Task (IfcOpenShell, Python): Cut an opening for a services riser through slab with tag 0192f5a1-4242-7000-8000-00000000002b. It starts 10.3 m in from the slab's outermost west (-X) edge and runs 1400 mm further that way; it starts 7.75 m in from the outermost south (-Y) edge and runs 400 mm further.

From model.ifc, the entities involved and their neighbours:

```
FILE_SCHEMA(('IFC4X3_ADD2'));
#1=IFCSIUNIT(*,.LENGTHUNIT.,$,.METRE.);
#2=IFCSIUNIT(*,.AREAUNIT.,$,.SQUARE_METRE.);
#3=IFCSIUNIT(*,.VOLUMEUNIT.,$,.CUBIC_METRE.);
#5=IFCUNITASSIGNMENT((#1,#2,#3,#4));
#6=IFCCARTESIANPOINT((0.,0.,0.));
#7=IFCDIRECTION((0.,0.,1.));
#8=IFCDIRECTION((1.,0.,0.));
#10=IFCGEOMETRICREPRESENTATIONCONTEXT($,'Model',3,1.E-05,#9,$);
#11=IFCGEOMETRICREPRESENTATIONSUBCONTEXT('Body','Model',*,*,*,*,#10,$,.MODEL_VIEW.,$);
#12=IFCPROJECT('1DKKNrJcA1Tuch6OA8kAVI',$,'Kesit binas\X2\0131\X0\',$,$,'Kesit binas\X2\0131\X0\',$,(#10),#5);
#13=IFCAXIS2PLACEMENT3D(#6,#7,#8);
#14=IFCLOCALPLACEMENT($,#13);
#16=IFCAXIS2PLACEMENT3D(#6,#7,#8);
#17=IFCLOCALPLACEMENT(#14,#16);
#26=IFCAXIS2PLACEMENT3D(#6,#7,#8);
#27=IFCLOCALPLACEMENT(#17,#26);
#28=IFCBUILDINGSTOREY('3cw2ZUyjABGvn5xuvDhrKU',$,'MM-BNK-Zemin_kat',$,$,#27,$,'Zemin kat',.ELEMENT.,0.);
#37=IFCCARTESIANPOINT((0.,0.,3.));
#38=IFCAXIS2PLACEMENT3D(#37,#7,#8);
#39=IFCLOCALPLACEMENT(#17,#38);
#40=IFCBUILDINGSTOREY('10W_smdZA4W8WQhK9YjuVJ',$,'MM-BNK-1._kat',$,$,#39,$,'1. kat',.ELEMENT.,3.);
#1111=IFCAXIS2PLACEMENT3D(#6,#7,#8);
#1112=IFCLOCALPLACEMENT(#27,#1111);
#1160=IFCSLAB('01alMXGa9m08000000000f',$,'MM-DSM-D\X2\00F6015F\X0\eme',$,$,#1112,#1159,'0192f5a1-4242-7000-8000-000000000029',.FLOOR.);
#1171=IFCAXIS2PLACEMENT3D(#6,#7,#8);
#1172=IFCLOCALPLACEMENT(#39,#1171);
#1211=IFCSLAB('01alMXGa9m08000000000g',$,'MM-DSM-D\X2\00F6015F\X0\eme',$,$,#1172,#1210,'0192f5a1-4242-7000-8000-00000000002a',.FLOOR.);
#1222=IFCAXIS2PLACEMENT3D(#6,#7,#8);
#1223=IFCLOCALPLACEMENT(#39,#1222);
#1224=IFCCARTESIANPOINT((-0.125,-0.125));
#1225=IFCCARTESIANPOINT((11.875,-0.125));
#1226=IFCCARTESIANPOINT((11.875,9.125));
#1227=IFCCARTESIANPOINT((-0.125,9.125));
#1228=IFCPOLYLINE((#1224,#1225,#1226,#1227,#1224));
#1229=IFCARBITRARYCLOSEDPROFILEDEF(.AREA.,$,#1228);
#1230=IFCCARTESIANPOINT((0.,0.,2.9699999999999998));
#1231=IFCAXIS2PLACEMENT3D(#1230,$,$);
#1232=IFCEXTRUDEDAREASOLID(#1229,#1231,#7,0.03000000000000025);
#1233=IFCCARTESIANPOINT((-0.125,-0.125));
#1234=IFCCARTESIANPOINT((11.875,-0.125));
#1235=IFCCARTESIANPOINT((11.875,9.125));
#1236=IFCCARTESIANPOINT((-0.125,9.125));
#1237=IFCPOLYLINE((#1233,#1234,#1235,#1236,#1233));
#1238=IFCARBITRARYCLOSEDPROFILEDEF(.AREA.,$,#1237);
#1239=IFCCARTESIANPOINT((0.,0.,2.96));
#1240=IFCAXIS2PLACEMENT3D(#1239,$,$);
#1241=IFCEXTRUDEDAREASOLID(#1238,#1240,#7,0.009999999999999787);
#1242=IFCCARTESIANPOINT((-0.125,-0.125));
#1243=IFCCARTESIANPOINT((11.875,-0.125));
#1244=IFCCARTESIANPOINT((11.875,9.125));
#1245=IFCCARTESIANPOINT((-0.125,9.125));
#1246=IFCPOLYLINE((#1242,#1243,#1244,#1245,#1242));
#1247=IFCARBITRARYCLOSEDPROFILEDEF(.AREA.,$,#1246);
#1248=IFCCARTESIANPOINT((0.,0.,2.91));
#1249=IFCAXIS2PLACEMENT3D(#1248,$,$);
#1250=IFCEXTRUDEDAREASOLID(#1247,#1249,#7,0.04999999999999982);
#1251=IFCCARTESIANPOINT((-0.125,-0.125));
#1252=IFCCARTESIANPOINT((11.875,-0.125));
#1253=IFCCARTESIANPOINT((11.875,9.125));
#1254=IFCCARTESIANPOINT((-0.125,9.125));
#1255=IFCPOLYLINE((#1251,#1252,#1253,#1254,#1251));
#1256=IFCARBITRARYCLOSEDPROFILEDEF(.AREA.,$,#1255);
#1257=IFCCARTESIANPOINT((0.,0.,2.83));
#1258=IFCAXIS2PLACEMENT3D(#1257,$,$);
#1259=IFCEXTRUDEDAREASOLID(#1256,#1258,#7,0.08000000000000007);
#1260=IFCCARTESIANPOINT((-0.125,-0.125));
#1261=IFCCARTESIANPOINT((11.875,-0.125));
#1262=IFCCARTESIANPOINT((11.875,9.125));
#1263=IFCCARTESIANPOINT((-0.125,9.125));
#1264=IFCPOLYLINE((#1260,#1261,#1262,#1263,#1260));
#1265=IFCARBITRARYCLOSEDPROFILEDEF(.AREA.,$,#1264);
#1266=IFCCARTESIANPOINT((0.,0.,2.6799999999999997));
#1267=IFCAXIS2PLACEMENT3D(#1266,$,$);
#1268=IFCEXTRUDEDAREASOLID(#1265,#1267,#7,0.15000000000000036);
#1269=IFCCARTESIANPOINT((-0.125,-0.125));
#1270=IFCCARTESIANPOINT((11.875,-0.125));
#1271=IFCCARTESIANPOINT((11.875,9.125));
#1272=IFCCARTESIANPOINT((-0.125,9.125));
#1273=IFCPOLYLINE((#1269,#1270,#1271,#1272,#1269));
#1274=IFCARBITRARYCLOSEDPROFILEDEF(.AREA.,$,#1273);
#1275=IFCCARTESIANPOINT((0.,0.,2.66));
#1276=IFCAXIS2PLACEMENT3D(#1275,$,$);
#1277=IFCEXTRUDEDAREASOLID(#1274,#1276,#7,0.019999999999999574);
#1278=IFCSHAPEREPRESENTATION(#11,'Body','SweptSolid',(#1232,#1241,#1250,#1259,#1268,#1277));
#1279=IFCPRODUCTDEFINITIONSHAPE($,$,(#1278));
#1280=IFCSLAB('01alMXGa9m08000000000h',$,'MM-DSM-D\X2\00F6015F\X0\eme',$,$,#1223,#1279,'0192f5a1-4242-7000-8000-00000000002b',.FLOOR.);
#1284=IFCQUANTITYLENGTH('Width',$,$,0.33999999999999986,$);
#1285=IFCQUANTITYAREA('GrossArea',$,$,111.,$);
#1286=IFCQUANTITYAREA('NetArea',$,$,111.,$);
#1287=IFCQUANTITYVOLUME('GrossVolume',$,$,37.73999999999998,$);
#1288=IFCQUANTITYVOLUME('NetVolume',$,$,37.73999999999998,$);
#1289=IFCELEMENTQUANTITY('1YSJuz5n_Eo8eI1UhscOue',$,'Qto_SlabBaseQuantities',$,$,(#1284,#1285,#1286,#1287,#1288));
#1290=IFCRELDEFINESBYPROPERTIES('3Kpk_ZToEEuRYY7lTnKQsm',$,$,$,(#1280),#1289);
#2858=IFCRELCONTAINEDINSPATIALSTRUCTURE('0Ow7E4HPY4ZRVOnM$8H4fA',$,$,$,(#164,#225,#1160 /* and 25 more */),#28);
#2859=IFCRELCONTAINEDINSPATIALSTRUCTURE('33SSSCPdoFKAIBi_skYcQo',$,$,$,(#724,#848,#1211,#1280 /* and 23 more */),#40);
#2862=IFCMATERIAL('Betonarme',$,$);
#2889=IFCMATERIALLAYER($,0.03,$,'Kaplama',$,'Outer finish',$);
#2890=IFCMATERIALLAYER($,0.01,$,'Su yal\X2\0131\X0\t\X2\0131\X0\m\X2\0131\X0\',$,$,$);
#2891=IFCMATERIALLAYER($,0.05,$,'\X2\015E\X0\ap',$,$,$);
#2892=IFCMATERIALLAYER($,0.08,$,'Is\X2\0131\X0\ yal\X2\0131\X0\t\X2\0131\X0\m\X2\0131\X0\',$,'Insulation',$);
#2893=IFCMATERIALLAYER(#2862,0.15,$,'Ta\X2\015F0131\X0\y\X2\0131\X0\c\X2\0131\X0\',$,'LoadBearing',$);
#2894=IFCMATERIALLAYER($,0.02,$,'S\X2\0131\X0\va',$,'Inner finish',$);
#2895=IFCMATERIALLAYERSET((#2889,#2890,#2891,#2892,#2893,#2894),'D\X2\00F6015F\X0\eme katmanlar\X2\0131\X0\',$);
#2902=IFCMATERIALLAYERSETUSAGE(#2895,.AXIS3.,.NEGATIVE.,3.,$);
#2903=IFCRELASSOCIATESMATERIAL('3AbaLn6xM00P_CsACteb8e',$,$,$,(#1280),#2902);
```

```python
import numpy as np
import ifcopenshell
import ifcopenshell.api.feature
import ifcopenshell.api.geometry
import ifcopenshell.api.pset
import ifcopenshell.api.root
import ifcopenshell.geom
import ifcopenshell.util.element
import ifcopenshell.util.placement
import ifcopenshell.util.representation
import ifcopenshell.util.shape
import ifcopenshell.util.unit

model = ifcopenshell.open("model.ifc")
unit_scale = ifcopenshell.util.unit.calculate_unit_scale(model)
area_scale = ifcopenshell.util.unit.calculate_unit_scale(model, "AREAUNIT")
volume_scale = ifcopenshell.util.unit.calculate_unit_scale(model, "VOLUMEUNIT")
settings = ifcopenshell.geom.settings()


def volume(element):
    """Net volume in cubic metres, openings subtracted."""
    shape = ifcopenshell.geom.create_shape(settings, element)
    return ifcopenshell.util.shape.get_volume(shape.geometry)


slab = model.by_guid("01alMXGa9m08000000000h")
before = volume(slab)

# Extent in the slab's own axes, in metres. The edges named are its -X and -Y sides.
slab_shape = ifcopenshell.geom.create_shape(settings, slab)
vertices = ifcopenshell.util.shape.get_vertices(slab_shape.geometry)
x_min, y_min, bottom = vertices.min(axis=0)
top = vertices[:, 2].max()

opening = ifcopenshell.api.root.create_entity(model, ifc_class="IfcOpeningElement", name="Services riser opening", predefined_type="OPENING")
context = ifcopenshell.util.representation.get_context(model, "Model", "Body", "MODEL_VIEW")
width, depth = 1.4, 0.4
outline = [(0.0, 0.0), (width, 0.0), (width, depth), (0.0, depth), (0.0, 0.0)]
# Overshoot both faces by 50 mm so the cut is clean.
shape = ifcopenshell.api.geometry.add_slab_representation(
    model, context=context, depth=top - bottom + 0.1, polyline=outline
)
ifcopenshell.api.geometry.assign_representation(model, product=opening, representation=shape)

matrix = ifcopenshell.util.placement.get_local_placement(slab.ObjectPlacement)
matrix[:, 3] = matrix @ np.append(np.array([x_min + 10.3, y_min + 7.75, bottom - 0.05]) / unit_scale, 1.0)
ifcopenshell.api.geometry.edit_object_placement(model, product=opening, matrix=matrix, is_si=False)
ifcopenshell.api.feature.add_feature(model, feature=opening, element=slab)

after = volume(slab)

# Update the slab's stored quantities.
qto = model.by_id(ifcopenshell.util.element.get_pset(slab, "Qto_SlabBaseQuantities", should_inherit=False)["id"])
ifcopenshell.api.pset.edit_qto(model, qto=qto, properties={
    "NetArea": after / (top - bottom) / area_scale,
    "NetVolume": after / volume_scale,
})

print(f"slab volume {before:.3f} -> {after:.3f} m3")

model.write("model-out.ifc")
```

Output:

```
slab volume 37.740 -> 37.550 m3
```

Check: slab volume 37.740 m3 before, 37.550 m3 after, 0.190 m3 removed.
